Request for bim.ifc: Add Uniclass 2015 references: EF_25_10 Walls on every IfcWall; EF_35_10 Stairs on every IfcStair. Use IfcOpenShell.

First a look at what the model holds.

```python
import ifcopenshell

model = ifcopenshell.open("bim.ifc")
print(model.schema)
print("classifications:", [c.Name for c in model.by_type("IfcClassification")])
for ifc_class in ("IfcDoor", "IfcRoof", "IfcStair", "IfcWall", "IfcWindow"):
    print(ifc_class, len(model.by_type(ifc_class)))
```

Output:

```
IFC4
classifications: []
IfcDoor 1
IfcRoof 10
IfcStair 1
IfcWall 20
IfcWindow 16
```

```python
import ifcopenshell
import ifcopenshell.api.classification

model = ifcopenshell.open("bim.ifc")

system = ifcopenshell.api.classification.add_classification(model, classification="Uniclass 2015")

codes = {
    "IfcWall": ("EF_25_10", "Walls"),
    "IfcStair": ("EF_35_10", "Stairs"),
}
for ifc_class, (code, name) in codes.items():
    products = model.by_type(ifc_class)
    ifcopenshell.api.classification.add_reference(
        model, products=products, classification=system, identification=code, name=name
    )
    print(code, len(products))

model.write("bim_rev.ifc")
```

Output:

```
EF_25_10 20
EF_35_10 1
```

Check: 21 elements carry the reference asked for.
